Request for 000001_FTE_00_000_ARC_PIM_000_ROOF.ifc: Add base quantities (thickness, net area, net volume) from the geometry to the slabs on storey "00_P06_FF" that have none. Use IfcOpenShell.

First a look at what the model holds.

```python
import ifcopenshell
import ifcopenshell.util.element
import ifcopenshell.util.unit

model = ifcopenshell.open("000001_FTE_00_000_ARC_PIM_000_ROOF.ifc")
print(model.schema)
for unit_type in ("LENGTHUNIT", "AREAUNIT", "VOLUMEUNIT"):
    print(unit_type, ifcopenshell.util.unit.calculate_unit_scale(model, unit_type))
storey = next(s for s in model.by_type("IfcBuildingStorey") if s.Name == "00_P06_FF")
slabs = [e for e in ifcopenshell.util.element.get_decomposition(storey) if e.is_a("IfcSlab")]
for e in sorted(slabs, key=lambda e: e.id()):
    print(e.id(), e.is_a(), e.Name, list(ifcopenshell.util.element.get_psets(e, qtos_only=True)), sep=" | ")
```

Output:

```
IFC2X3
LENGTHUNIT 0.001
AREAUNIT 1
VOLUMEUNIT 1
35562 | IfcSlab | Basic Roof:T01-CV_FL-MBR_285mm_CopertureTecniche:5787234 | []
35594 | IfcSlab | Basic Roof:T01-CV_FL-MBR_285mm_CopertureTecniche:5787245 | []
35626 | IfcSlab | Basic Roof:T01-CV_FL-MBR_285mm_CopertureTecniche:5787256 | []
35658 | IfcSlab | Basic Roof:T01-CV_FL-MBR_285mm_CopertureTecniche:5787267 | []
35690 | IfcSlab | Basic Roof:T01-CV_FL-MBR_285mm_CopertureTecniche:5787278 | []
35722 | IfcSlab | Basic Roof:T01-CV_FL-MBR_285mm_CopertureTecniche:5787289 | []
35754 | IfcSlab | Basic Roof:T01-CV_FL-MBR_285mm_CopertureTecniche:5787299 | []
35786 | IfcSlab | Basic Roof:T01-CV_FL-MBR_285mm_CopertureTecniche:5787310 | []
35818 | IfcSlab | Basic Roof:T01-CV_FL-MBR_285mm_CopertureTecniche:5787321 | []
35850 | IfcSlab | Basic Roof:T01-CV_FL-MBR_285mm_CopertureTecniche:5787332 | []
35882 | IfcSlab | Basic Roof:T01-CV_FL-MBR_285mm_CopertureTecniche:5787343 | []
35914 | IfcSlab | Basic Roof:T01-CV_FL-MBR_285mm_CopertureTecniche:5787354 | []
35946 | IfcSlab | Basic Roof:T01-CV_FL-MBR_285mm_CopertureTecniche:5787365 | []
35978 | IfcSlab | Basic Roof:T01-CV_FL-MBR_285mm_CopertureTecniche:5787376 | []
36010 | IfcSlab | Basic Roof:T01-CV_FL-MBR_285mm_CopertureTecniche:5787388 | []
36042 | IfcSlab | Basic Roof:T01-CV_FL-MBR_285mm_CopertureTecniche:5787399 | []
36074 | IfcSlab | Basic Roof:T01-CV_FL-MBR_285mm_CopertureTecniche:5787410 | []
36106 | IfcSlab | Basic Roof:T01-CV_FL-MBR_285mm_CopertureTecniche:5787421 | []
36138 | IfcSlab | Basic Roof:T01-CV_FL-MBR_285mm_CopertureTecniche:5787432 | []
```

```python
import ifcopenshell
import ifcopenshell.api.pset
import ifcopenshell.geom
import ifcopenshell.util.element
import ifcopenshell.util.shape
import ifcopenshell.util.unit

model = ifcopenshell.open("000001_FTE_00_000_ARC_PIM_000_ROOF.ifc")
unit_scale = ifcopenshell.util.unit.calculate_unit_scale(model)
area_scale = ifcopenshell.util.unit.calculate_unit_scale(model, "AREAUNIT")
volume_scale = ifcopenshell.util.unit.calculate_unit_scale(model, "VOLUMEUNIT")
settings = ifcopenshell.geom.settings()

storey = next(s for s in model.by_type("IfcBuildingStorey") if s.Name == "00_P06_FF")
slabs = [e for e in ifcopenshell.util.element.get_decomposition(storey) if e.is_a("IfcSlab")]

for e in sorted(slabs, key=lambda e: e.id()):
    if ifcopenshell.util.element.get_psets(e, qtos_only=True, should_inherit=False):
        continue
    # Geometry comes back in metres, in the element's own axes.
    shape = ifcopenshell.geom.create_shape(settings, e)
    values = {
        "Width": ifcopenshell.util.shape.get_z(shape.geometry) / unit_scale,
        "NetArea": ifcopenshell.util.shape.get_footprint_area(shape.geometry) / area_scale,
        "NetVolume": ifcopenshell.util.shape.get_volume(shape.geometry) / volume_scale,
    }
    qto = ifcopenshell.api.pset.add_qto(model, product=e, name="BaseQuantities")
    ifcopenshell.api.pset.edit_qto(model, qto=qto, properties=values)
    print(e.id(), {k: round(v, 3) for k, v in values.items()})

model.write("000001_FTE_00_000_ARC_PIM_000_ROOF_edited.ifc")
```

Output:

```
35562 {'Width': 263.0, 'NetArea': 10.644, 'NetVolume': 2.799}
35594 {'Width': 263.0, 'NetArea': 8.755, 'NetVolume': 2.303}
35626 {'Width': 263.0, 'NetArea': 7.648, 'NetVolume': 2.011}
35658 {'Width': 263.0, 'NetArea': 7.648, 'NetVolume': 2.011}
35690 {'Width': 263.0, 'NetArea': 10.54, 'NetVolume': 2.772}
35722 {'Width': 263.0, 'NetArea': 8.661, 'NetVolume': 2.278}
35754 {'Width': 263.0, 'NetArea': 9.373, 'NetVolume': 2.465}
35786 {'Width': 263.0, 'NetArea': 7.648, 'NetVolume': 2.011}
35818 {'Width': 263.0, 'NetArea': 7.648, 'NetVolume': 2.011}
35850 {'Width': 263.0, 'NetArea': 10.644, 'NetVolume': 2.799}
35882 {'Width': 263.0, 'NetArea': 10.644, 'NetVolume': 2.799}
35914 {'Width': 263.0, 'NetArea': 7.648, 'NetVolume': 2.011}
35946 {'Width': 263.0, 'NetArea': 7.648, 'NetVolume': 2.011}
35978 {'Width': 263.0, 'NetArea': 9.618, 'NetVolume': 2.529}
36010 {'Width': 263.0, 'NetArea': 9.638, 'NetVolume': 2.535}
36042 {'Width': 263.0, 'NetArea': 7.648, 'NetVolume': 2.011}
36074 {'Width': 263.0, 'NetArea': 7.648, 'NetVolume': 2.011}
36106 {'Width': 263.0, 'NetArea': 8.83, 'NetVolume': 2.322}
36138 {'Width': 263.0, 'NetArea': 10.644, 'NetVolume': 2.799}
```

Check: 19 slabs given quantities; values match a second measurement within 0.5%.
